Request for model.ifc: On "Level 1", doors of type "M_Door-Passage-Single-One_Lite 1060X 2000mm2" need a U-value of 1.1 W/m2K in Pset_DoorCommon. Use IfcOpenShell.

First a look at what the model holds.

```python
import ifcopenshell
import ifcopenshell.util.element

model = ifcopenshell.open("model.ifc")
print(model.schema)
storey = next(s for s in model.by_type("IfcBuildingStorey") if s.Name == "Level 1")
doors = [e for e in ifcopenshell.util.element.get_decomposition(storey) if e.is_a("IfcDoor")]
seen = {}
for e in doors:
    element_type = ifcopenshell.util.element.get_type(e)
    key = (element_type.Name if element_type != e and element_type else None, ifcopenshell.util.element.get_pset(e, "Pset_DoorCommon", "ThermalTransmittance"))
    seen[key] = seen.get(key, 0) + 1
for (name, value), count in sorted(seen.items(), key=str):
    print(count, "x", name, "|", value)
```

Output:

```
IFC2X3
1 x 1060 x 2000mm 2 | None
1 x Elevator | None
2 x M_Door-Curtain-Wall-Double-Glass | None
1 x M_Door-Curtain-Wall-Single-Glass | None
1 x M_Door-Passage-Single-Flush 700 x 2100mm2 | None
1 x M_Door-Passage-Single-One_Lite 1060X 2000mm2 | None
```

```python
import ifcopenshell
import ifcopenshell.api.pset
import ifcopenshell.util.element

model = ifcopenshell.open("model.ifc")

storey = next(s for s in model.by_type("IfcBuildingStorey") if s.Name == "Level 1")
doors = [e for e in ifcopenshell.util.element.get_decomposition(storey) if e.is_a("IfcDoor")]

count = 0
for e in doors:
    element_type = ifcopenshell.util.element.get_type(e)
    if element_type in (None, e) or element_type.Name != "M_Door-Passage-Single-One_Lite 1060X 2000mm2":
        continue
    # add_pset returns the element's existing set when there is one.
    pset = ifcopenshell.api.pset.add_pset(model, product=e, name="Pset_DoorCommon")
    ifcopenshell.api.pset.edit_pset(model, pset=pset, properties={"ThermalTransmittance": 1.1})
    count += 1

print(count, "doors updated")

model.write("model_rev.ifc")
```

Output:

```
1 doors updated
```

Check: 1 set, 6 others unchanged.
